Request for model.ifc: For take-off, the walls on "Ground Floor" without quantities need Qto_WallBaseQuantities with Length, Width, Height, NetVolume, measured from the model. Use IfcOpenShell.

First a look at what the model holds.

```python
import ifcopenshell
import ifcopenshell.util.element
import ifcopenshell.util.unit

model = ifcopenshell.open("model.ifc")
print(model.schema)
for unit_type in ("LENGTHUNIT", "AREAUNIT", "VOLUMEUNIT"):
    print(unit_type, ifcopenshell.util.unit.calculate_unit_scale(model, unit_type))
storey = next(s for s in model.by_type("IfcBuildingStorey") if s.Name == "Ground Floor")
walls = [e for e in ifcopenshell.util.element.get_decomposition(storey) if e.is_a("IfcWall")]
for e in sorted(walls, key=lambda e: e.id()):
    print(e.id(), e.is_a(), e.Name, list(ifcopenshell.util.element.get_psets(e, qtos_only=True)), sep=" | ")
```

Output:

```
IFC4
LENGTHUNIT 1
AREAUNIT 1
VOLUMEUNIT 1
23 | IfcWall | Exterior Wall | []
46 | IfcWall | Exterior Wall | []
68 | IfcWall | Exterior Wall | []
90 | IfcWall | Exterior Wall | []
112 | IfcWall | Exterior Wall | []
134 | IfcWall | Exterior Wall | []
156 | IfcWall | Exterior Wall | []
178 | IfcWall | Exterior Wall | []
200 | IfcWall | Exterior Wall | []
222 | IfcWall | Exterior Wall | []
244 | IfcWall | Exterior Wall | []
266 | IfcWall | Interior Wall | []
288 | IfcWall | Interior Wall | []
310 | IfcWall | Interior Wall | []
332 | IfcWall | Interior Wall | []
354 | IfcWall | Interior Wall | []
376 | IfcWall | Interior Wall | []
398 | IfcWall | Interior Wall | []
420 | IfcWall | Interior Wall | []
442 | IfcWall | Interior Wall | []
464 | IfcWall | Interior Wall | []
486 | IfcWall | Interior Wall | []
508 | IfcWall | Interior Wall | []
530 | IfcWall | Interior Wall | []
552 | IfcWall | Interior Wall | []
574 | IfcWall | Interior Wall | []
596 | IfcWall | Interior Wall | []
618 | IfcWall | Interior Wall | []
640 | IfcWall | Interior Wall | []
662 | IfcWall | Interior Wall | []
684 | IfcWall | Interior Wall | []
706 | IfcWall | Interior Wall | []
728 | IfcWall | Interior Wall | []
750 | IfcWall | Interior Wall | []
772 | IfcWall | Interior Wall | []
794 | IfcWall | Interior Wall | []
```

```python
import ifcopenshell
import ifcopenshell.api.pset
import ifcopenshell.geom
import ifcopenshell.util.element
import ifcopenshell.util.shape
import ifcopenshell.util.unit

model = ifcopenshell.open("model.ifc")
unit_scale = ifcopenshell.util.unit.calculate_unit_scale(model)
volume_scale = ifcopenshell.util.unit.calculate_unit_scale(model, "VOLUMEUNIT")
settings = ifcopenshell.geom.settings()

storey = next(s for s in model.by_type("IfcBuildingStorey") if s.Name == "Ground Floor")
walls = [e for e in ifcopenshell.util.element.get_decomposition(storey) if e.is_a("IfcWall")]

for e in sorted(walls, key=lambda e: e.id()):
    if ifcopenshell.util.element.get_psets(e, qtos_only=True, should_inherit=False):
        continue
    # Geometry comes back in metres, in the element's own axes.
    shape = ifcopenshell.geom.create_shape(settings, e)
    values = {
        "Length": ifcopenshell.util.shape.get_x(shape.geometry) / unit_scale,
        "Width": ifcopenshell.util.shape.get_y(shape.geometry) / unit_scale,
        "Height": ifcopenshell.util.shape.get_z(shape.geometry) / unit_scale,
        "NetVolume": ifcopenshell.util.shape.get_volume(shape.geometry) / volume_scale,
    }
    qto = ifcopenshell.api.pset.add_qto(model, product=e, name="Qto_WallBaseQuantities")
    ifcopenshell.api.pset.edit_qto(model, qto=qto, properties=values)
    print(e.id(), {k: round(v, 3) for k, v in values.items()})

model.write("model-out.ifc")
```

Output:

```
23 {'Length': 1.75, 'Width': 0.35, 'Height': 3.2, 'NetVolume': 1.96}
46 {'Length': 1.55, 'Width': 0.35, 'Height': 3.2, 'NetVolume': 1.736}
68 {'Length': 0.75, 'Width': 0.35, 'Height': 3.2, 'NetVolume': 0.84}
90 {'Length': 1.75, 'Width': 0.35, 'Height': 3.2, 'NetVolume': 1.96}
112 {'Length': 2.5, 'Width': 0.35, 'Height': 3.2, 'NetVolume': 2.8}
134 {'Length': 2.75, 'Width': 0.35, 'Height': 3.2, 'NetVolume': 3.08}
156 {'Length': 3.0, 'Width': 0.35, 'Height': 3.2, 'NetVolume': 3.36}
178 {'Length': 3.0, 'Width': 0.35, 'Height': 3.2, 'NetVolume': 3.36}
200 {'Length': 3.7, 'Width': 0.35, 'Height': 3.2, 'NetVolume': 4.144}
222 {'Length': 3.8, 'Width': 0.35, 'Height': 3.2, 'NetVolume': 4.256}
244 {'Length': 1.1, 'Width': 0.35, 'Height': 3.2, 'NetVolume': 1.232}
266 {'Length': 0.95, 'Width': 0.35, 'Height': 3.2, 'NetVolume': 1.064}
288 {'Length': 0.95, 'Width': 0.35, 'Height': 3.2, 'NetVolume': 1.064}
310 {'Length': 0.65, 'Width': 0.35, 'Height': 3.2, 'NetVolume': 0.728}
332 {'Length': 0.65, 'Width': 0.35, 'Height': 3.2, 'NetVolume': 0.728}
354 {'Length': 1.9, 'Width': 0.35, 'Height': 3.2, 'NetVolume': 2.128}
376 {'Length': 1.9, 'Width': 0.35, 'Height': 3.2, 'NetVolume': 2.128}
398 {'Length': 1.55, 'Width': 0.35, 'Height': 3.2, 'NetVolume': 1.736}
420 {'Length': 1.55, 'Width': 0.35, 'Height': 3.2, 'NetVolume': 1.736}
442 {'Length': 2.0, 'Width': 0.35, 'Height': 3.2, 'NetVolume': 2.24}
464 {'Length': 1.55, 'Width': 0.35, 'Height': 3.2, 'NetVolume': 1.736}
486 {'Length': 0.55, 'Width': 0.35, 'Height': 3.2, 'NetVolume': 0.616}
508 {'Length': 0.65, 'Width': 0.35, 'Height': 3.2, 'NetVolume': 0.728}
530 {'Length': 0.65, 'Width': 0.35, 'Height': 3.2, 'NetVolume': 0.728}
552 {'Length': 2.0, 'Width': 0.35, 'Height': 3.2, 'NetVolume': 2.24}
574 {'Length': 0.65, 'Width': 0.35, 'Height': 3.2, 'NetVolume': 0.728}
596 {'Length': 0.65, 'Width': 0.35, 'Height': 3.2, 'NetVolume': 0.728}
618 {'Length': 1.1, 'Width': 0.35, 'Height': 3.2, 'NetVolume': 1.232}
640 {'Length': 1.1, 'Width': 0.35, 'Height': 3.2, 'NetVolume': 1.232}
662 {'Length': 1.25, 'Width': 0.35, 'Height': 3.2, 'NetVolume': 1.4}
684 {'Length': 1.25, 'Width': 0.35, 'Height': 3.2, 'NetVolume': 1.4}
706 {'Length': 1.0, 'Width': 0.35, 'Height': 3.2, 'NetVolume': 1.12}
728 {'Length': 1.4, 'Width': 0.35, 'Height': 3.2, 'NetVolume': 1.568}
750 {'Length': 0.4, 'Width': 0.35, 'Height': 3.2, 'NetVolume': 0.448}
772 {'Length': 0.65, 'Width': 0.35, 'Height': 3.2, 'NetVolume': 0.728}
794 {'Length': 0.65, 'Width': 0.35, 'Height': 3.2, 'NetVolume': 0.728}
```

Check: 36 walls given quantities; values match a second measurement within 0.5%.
